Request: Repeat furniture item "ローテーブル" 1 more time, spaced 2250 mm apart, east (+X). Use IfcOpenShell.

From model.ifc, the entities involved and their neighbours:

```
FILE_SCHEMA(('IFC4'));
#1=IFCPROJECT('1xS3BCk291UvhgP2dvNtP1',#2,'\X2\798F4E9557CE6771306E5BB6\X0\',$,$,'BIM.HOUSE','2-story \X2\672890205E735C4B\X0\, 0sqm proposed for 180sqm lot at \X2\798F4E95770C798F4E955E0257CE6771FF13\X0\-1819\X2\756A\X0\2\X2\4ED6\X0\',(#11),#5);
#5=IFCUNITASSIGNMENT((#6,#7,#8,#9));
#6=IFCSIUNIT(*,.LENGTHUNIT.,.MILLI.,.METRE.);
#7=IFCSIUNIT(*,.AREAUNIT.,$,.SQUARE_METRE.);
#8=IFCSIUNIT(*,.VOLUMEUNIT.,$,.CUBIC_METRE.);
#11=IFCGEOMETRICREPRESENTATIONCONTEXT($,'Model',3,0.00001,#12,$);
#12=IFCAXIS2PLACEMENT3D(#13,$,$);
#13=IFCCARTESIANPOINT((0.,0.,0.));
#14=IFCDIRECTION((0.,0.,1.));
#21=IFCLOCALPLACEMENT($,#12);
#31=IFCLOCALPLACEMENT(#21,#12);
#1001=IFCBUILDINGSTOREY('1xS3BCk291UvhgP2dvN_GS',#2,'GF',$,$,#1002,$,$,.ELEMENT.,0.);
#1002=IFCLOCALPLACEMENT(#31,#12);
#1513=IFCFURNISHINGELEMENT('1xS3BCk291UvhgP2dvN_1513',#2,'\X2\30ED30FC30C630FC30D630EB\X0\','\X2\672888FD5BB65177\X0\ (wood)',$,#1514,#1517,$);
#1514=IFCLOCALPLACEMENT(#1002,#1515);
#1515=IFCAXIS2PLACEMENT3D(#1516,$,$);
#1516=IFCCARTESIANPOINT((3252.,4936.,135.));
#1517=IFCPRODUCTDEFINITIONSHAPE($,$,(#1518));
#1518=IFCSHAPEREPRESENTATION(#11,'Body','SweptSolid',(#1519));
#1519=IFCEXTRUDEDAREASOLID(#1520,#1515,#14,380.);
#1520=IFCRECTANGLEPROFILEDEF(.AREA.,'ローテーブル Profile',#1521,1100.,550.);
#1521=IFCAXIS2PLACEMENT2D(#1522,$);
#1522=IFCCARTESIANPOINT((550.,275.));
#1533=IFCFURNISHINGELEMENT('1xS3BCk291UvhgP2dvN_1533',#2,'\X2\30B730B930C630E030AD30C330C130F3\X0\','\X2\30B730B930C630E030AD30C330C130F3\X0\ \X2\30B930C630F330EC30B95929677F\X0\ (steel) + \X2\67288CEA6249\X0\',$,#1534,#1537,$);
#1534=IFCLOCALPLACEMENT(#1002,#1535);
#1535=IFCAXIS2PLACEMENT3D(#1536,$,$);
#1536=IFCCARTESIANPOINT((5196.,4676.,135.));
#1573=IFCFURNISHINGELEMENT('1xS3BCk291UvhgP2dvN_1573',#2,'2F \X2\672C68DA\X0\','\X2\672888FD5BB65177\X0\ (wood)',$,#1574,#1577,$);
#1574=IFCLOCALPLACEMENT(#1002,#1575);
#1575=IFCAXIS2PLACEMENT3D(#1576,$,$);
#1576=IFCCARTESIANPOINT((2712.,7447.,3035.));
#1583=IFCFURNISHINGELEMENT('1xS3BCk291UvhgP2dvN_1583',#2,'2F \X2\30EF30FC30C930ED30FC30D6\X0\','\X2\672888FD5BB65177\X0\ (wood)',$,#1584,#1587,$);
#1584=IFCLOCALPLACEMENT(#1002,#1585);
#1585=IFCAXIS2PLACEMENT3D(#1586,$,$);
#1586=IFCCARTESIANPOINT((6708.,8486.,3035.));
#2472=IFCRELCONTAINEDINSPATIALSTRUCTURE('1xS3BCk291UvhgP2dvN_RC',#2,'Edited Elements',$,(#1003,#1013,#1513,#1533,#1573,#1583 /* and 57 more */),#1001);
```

```python
import numpy as np
import ifcopenshell
import ifcopenshell.api.geometry
import ifcopenshell.api.root
import ifcopenshell.util.element
import ifcopenshell.util.placement
import ifcopenshell.util.unit

model = ifcopenshell.open("model.ifc")
unit_scale = ifcopenshell.util.unit.calculate_unit_scale(model)


def reuse_history(source, copy):
    """copy_class also copies each property set's owner history, people and application; keep the originals."""
    for rel in copy.IsDefinedBy:
        if rel.is_a("IfcRelDefinesByProperties") and (history := rel.RelatingPropertyDefinition.OwnerHistory):
            rel.RelatingPropertyDefinition.OwnerHistory = source.OwnerHistory
            ifcopenshell.util.element.remove_deep2(model, history)


source = model.by_guid("1xS3BCk291UvhgP2dvN_1513")
base = ifcopenshell.util.placement.get_local_placement(source.ObjectPlacement)
step = np.array([1.0, 0.0, 0.0]) * 2.25 / unit_scale

for i in range(1, 2):
    copy = ifcopenshell.api.root.copy_class(model, product=source)
    copy.Representation = ifcopenshell.util.element.copy_deep(
        model, source.Representation, exclude=["IfcGeometricRepresentationContext", "IfcRepresentationMap"]
    )
    reuse_history(source, copy)
    matrix = base.copy()
    matrix[:3, 3] += i * step
    print("added at", matrix[:3, 3].round(3) + 0.0)
    ifcopenshell.api.geometry.edit_object_placement(model, product=copy, matrix=matrix, is_si=False)

model.write("model_updated.ifc")
```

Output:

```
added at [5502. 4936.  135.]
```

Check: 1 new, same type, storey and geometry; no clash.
